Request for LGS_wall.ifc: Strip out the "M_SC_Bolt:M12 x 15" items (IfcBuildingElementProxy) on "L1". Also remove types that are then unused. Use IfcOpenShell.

First a look at what the model holds.

```python
import ifcopenshell
import ifcopenshell.util.element

model = ifcopenshell.open("LGS_wall.ifc")
print(model.schema)
storey = next(s for s in model.by_type("IfcBuildingStorey") if s.Name == "L1")
proxies = [e for e in ifcopenshell.util.element.get_decomposition(storey) if e.is_a("IfcBuildingElementProxy")]
seen = {}
for e in proxies:
    element_type = ifcopenshell.util.element.get_type(e)
    name = element_type.Name if element_type not in (None, e) else None
    seen[name] = seen.get(name, 0) + 1
for name, count in sorted(seen.items(), key=str):
    print(count, "x", name)
```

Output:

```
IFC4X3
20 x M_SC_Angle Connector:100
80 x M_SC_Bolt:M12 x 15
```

```python
import ifcopenshell
import ifcopenshell.api.root
import ifcopenshell.util.element

model = ifcopenshell.open("LGS_wall.ifc")

storey = next(s for s in model.by_type("IfcBuildingStorey") if s.Name == "L1")
proxies = [e for e in ifcopenshell.util.element.get_decomposition(storey) if e.is_a("IfcBuildingElementProxy")]
targets = [e for e in proxies if (t := ifcopenshell.util.element.get_type(e)) not in (None, e) and t.Name == "M_SC_Bolt:M12 x 15"]
types = {ifcopenshell.util.element.get_type(e) for e in targets} - {None, *targets}

for e in targets:
    ifcopenshell.api.root.remove_product(model, product=e)
print(len(targets), "removed")

unused = [t for t in types if not ifcopenshell.util.element.get_types(t)]
for t in unused:
    ifcopenshell.api.root.remove_product(model, product=t)
print(len(unused), "unused types removed")

model.write("LGS_wall_v2.ifc")
```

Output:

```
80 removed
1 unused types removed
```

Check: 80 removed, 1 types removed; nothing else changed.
